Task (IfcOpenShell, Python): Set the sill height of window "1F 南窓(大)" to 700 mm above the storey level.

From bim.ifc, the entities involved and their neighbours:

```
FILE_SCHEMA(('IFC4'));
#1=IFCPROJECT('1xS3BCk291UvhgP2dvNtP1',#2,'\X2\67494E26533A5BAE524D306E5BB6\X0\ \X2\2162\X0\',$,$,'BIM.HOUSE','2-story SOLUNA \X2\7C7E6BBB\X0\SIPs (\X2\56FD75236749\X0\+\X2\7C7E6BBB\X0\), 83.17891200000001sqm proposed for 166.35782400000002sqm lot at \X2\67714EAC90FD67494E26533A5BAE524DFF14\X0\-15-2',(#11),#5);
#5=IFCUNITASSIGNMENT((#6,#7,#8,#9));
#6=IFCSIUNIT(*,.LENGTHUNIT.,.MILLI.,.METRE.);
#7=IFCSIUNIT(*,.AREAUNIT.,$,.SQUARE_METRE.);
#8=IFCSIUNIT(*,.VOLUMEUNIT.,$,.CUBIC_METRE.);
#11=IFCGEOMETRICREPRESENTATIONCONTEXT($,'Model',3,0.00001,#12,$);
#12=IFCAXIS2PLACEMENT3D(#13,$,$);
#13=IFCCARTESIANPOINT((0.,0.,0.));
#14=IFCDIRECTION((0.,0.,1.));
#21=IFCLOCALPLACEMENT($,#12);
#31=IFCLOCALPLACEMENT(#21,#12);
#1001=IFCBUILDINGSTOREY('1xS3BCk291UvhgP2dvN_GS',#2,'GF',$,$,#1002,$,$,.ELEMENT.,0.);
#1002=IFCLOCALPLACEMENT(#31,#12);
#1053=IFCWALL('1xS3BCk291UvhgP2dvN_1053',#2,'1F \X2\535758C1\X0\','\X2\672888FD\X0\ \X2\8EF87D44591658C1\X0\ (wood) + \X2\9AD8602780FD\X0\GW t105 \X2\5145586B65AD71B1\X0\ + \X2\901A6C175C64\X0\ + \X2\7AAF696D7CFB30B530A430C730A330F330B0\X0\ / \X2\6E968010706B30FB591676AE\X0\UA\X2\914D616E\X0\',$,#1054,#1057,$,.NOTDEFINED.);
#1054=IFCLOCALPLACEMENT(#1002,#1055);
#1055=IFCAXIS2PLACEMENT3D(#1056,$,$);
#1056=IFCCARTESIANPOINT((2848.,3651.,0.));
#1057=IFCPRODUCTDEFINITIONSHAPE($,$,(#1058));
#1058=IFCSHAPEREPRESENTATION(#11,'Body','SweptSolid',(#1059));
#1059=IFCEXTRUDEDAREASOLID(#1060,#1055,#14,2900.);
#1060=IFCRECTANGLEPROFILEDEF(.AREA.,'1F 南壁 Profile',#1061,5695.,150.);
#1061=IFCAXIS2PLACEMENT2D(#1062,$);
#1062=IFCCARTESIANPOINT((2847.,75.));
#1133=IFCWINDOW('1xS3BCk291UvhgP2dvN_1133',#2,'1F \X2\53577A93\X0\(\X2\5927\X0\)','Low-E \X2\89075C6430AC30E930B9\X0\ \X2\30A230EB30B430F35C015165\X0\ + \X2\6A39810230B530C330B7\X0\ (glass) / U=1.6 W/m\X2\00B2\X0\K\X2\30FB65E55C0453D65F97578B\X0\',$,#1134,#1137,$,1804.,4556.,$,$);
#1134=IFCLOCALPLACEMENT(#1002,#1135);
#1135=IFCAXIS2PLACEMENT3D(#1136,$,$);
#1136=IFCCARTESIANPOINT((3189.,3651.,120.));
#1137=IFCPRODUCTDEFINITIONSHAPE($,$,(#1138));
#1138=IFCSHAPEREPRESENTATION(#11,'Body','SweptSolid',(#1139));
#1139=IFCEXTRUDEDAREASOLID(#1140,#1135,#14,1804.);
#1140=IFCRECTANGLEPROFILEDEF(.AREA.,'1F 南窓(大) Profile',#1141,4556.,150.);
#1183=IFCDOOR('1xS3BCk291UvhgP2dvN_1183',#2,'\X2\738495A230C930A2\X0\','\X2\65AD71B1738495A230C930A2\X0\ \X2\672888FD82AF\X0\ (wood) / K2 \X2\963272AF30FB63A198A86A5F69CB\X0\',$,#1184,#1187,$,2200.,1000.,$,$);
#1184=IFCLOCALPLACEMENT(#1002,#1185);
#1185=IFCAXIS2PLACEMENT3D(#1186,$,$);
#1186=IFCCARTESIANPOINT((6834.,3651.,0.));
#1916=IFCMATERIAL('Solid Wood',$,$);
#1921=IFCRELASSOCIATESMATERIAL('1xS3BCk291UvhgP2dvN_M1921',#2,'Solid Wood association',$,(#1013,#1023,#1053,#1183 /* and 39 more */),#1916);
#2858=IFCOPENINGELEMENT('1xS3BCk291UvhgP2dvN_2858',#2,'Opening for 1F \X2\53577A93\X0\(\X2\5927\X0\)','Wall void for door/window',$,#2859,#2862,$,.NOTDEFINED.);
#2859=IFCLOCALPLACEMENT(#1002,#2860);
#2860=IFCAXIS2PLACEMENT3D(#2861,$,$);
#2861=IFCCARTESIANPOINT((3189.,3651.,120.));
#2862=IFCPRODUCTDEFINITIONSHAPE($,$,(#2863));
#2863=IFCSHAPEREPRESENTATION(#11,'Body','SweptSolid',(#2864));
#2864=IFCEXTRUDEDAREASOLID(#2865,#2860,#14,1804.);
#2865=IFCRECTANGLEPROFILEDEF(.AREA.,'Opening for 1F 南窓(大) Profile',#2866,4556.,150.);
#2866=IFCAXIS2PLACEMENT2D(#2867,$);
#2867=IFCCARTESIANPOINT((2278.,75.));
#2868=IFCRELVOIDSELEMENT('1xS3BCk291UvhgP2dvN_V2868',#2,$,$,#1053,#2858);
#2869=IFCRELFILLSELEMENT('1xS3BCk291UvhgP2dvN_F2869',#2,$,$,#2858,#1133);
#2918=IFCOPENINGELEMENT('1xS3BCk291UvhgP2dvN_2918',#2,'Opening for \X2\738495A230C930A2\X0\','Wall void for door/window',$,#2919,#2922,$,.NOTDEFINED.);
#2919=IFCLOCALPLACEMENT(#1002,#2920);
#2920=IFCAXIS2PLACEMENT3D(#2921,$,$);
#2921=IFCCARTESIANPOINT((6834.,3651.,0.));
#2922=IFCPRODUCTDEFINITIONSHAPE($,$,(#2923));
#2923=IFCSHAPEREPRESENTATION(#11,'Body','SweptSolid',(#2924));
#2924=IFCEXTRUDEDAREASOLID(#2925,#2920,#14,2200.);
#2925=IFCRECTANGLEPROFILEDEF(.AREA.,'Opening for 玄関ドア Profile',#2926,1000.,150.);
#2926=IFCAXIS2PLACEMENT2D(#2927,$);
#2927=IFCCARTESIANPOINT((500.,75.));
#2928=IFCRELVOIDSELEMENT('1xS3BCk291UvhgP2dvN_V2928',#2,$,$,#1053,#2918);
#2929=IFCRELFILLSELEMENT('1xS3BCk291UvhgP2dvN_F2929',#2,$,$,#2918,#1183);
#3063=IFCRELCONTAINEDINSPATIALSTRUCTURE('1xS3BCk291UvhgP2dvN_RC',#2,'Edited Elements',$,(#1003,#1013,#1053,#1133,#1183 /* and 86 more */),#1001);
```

```python
import numpy as np
import ifcopenshell
import ifcopenshell.api.geometry
import ifcopenshell.geom
import ifcopenshell.util.element
import ifcopenshell.util.placement
import ifcopenshell.util.shape
import ifcopenshell.util.unit

model = ifcopenshell.open("bim.ifc")
unit_scale = ifcopenshell.util.unit.calculate_unit_scale(model)

window = model.by_id(1133)
opening = window.FillsVoids[0].RelatingOpeningElement
storey = ifcopenshell.util.element.get_container(window, ifc_class="IfcBuildingStorey")
level = ifcopenshell.util.placement.get_local_placement(storey.ObjectPlacement)[2, 3]

# The opening's origin need not be at the sill, so measure its lowest point.
shape = ifcopenshell.geom.create_shape(ifcopenshell.geom.settings(), opening)
bottom = ifcopenshell.util.shape.get_shape_bottom_elevation(shape, shape.geometry) / unit_scale
dz = level + 700.0 - bottom

shift = np.array([0.0, 0.0, dz])
# The window is not placed relative to its opening, so move both.
for product in (opening, window):
    matrix = ifcopenshell.util.placement.get_local_placement(product.ObjectPlacement)
    matrix[:3, 3] += shift
    ifcopenshell.api.geometry.edit_object_placement(model, product=product, matrix=matrix, is_si=False)

print(f"moved by {dz * unit_scale:+.3f} m")

model.write("bim_rev.ifc")
```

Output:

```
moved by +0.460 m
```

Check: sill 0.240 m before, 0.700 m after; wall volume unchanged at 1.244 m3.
